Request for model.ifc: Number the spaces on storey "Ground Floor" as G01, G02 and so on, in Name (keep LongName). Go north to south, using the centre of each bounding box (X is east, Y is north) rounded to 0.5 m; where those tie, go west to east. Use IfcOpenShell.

First a look at what the model holds.

```python
import ifcopenshell
import ifcopenshell.util.element
import ifcopenshell.util.placement

model = ifcopenshell.open("model.ifc")
print(model.schema)
storey = next(s for s in model.by_type("IfcBuildingStorey") if s.Name == "Ground Floor")
spaces = [e for e in ifcopenshell.util.element.get_decomposition(storey) if e.is_a("IfcSpace")]
for e in sorted(spaces, key=lambda e: e.id()):
    origin = ifcopenshell.util.placement.get_local_placement(e.ObjectPlacement)[:3, 3]
    print(e.id(), e.Name, e.LongName, origin.round(2) + 0.0, sep=" | ")
```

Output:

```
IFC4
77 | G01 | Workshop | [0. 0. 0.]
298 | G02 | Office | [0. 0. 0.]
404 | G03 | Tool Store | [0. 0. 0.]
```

```python
import ifcopenshell
import ifcopenshell.geom
import ifcopenshell.util.element
import ifcopenshell.util.shape

model = ifcopenshell.open("model.ifc")
settings = ifcopenshell.geom.settings()
settings.set("use-world-coords", True)


def centre(element):
    shape = ifcopenshell.geom.create_shape(settings, element)
    return ifcopenshell.util.shape.get_bbox_centroid(shape.geometry)


storey = next(s for s in model.by_type("IfcBuildingStorey") if s.Name == "Ground Floor")
spaces = [e for e in ifcopenshell.util.element.get_decomposition(storey) if e.is_a("IfcSpace")]

# Insertion points can sit at a corner or the storey origin, so sort by the geometry (in metres).
centres = {e: centre(e) for e in spaces}
spaces.sort(key=lambda e: (-round(centres[e][1] / 0.5), centres[e][0]))

for i, e in enumerate(spaces, start=1):
    number = f"G{i:02d}"
    e.Name = number
    print(e.id(), number)

model.write("model_updated.ifc")
```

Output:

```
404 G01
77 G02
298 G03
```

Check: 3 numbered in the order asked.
